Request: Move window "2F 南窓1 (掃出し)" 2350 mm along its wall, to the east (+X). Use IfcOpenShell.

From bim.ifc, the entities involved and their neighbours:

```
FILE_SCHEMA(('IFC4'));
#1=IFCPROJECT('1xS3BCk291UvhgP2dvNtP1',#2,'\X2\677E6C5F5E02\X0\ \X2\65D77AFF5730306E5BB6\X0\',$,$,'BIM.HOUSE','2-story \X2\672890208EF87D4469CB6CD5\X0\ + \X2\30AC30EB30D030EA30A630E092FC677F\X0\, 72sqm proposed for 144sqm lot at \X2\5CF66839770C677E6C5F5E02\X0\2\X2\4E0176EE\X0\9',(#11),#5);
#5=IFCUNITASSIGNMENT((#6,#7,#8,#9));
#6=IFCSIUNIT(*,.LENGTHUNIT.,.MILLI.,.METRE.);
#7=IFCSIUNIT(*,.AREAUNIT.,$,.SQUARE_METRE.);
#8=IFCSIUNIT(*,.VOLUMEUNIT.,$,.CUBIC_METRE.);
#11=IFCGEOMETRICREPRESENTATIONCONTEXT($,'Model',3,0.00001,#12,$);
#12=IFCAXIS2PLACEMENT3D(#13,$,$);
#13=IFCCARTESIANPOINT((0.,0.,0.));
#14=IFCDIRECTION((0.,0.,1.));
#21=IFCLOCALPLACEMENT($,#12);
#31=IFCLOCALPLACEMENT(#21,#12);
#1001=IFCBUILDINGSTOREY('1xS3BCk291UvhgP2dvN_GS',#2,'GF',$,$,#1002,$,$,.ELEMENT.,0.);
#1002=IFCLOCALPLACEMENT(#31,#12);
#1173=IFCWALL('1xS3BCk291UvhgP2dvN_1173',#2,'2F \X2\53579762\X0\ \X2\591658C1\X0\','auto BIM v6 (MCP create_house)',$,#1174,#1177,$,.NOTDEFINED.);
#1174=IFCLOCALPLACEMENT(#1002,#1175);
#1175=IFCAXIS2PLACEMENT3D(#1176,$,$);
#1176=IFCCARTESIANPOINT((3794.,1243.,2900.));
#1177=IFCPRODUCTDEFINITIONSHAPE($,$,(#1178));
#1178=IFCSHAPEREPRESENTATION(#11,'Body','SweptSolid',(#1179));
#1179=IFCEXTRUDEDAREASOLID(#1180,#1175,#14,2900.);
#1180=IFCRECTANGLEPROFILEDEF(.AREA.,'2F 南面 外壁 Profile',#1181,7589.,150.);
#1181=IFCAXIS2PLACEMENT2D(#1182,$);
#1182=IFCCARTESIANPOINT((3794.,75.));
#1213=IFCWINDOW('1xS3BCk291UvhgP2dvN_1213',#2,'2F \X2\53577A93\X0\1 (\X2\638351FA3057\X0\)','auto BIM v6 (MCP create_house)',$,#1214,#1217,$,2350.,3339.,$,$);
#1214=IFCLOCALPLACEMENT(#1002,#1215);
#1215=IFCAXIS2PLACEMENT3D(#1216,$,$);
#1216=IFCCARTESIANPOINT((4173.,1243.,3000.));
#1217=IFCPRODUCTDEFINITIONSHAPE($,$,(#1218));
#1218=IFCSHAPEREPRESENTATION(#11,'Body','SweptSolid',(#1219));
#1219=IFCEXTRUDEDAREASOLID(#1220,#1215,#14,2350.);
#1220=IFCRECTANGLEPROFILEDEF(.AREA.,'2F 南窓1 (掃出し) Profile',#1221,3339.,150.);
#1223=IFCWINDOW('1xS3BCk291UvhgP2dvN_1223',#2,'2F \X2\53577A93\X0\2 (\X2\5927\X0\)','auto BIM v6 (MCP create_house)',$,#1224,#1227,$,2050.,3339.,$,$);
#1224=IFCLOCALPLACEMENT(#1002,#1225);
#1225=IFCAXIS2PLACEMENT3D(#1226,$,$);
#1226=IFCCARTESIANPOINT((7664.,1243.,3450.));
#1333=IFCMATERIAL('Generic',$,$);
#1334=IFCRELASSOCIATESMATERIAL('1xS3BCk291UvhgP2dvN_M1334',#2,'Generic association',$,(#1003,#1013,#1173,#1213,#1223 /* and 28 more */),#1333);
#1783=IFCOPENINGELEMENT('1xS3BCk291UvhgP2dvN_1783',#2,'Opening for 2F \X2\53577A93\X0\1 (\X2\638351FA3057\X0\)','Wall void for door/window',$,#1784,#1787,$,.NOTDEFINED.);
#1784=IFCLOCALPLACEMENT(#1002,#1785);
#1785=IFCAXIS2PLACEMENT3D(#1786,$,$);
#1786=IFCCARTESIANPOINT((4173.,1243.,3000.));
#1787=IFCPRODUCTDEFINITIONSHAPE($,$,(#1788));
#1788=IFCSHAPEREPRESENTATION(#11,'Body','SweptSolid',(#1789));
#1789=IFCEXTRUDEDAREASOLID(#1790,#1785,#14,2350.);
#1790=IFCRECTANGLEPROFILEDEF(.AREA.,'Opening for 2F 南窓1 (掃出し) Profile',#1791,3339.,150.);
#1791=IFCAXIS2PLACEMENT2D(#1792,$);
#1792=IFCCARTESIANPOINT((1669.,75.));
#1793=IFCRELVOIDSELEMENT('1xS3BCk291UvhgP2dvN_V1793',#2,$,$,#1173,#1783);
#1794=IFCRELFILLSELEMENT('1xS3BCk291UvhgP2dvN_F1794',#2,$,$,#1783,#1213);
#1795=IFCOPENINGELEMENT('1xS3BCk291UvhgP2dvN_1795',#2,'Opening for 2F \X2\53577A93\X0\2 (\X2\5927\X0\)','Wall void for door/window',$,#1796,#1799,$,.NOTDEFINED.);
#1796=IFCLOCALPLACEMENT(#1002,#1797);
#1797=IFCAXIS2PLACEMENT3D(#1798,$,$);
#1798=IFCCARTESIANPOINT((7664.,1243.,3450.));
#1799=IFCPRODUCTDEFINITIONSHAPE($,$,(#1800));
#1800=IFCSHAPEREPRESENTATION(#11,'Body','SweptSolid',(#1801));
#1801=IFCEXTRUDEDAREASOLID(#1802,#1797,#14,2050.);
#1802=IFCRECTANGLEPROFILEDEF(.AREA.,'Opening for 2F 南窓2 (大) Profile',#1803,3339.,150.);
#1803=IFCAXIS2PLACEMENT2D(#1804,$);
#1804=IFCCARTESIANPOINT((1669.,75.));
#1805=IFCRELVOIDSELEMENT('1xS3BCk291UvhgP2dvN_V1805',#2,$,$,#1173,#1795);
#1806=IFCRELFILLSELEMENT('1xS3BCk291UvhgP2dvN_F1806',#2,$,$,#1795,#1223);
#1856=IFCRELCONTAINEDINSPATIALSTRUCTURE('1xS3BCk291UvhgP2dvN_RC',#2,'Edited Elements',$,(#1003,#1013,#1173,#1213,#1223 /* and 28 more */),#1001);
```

```python
import ifcopenshell
import ifcopenshell.api.geometry
import ifcopenshell.util.placement

model = ifcopenshell.open("bim.ifc")

window = model.by_guid("1xS3BCk291UvhgP2dvN_1213")
opening = window.FillsVoids[0].RelatingOpeningElement
wall = opening.VoidsElements[0].RelatingBuildingElement

wall_matrix = ifcopenshell.util.placement.get_local_placement(wall.ObjectPlacement)
shift = wall_matrix[:3, 0] * 2350.0
before = ifcopenshell.util.placement.get_local_placement(window.ObjectPlacement)[:3, 3].copy()

# The window is not placed relative to its opening, so move both.
for product in (opening, window):
    matrix = ifcopenshell.util.placement.get_local_placement(product.ObjectPlacement)
    matrix[:3, 3] += shift
    ifcopenshell.api.geometry.edit_object_placement(model, product=product, matrix=matrix, is_si=False)

after = ifcopenshell.util.placement.get_local_placement(window.ObjectPlacement)[:3, 3]
print("window moved by", (after - before).round(3) + 0.0)

model.write("bim_rev.ifc")
```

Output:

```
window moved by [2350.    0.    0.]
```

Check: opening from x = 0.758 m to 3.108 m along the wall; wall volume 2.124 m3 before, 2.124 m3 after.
